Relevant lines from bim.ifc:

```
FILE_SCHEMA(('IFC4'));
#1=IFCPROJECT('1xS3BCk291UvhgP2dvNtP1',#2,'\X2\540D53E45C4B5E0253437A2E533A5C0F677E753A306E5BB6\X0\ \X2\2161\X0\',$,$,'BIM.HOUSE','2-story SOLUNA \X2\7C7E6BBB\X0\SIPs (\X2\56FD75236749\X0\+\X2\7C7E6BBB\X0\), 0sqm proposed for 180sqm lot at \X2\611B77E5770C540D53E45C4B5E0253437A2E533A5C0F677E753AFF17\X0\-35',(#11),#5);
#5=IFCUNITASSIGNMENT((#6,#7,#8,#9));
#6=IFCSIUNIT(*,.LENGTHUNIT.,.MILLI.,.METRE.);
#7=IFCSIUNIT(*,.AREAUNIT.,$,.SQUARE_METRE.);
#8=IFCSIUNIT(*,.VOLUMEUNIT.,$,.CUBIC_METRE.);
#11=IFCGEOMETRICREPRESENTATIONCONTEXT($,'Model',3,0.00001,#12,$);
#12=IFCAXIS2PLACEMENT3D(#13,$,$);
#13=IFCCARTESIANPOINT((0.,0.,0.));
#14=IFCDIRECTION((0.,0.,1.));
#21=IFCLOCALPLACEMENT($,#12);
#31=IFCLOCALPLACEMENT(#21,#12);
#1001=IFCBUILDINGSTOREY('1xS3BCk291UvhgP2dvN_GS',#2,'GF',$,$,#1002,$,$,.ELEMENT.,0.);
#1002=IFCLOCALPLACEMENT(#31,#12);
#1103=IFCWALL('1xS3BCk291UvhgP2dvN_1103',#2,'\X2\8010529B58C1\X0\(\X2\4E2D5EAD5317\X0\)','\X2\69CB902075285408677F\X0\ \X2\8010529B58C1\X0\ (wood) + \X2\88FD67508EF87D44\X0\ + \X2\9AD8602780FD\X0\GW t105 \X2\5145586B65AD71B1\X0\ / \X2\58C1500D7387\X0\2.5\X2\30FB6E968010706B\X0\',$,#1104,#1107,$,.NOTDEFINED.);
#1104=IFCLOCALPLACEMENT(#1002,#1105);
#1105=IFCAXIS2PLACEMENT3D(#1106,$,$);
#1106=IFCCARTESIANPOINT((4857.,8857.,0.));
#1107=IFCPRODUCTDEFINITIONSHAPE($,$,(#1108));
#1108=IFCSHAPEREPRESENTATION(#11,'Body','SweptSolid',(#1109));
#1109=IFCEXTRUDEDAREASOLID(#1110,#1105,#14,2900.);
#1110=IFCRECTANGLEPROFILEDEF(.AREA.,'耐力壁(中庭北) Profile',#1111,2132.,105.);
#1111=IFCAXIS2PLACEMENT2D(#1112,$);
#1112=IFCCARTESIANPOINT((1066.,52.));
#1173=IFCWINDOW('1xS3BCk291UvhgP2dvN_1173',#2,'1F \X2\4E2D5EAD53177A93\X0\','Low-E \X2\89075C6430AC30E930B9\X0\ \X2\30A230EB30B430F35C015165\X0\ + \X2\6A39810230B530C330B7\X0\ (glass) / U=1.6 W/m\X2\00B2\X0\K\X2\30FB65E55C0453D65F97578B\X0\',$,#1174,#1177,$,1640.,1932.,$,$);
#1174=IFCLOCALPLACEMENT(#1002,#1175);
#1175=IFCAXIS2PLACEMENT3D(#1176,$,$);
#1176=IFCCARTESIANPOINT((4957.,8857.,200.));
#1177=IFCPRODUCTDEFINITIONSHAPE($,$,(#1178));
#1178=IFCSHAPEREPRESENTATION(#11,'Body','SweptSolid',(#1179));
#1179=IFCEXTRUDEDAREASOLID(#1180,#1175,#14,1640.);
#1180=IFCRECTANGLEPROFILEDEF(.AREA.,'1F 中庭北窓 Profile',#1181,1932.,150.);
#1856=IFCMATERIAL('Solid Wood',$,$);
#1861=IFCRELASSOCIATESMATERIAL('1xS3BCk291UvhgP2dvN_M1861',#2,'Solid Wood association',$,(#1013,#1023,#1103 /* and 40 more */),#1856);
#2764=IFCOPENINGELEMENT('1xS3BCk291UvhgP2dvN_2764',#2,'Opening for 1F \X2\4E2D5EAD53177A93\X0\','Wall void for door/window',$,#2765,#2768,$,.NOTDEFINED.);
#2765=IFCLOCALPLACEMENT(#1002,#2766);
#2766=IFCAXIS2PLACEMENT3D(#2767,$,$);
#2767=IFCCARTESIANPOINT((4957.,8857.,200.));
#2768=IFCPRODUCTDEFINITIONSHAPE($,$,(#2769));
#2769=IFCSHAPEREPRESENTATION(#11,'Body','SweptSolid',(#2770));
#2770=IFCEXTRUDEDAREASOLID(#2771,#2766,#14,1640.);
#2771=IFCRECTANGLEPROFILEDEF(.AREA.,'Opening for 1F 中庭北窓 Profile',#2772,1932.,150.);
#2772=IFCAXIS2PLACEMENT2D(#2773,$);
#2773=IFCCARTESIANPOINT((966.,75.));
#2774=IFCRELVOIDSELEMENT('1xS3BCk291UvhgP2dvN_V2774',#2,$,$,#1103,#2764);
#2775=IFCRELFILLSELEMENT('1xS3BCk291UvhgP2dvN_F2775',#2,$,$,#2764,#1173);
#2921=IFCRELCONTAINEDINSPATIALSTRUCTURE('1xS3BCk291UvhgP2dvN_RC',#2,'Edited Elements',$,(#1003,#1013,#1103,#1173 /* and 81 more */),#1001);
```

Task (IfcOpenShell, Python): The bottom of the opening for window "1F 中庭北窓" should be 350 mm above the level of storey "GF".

```python
import numpy as np
import ifcopenshell
import ifcopenshell.api.geometry
import ifcopenshell.geom
import ifcopenshell.util.element
import ifcopenshell.util.placement
import ifcopenshell.util.shape
import ifcopenshell.util.unit

model = ifcopenshell.open("bim.ifc")
unit_scale = ifcopenshell.util.unit.calculate_unit_scale(model)

window = model.by_guid("1xS3BCk291UvhgP2dvN_1173")
opening = window.FillsVoids[0].RelatingOpeningElement
storey = ifcopenshell.util.element.get_container(window, ifc_class="IfcBuildingStorey")
level = ifcopenshell.util.placement.get_local_placement(storey.ObjectPlacement)[2, 3]

# The opening's origin need not be at the sill, so measure its lowest point.
shape = ifcopenshell.geom.create_shape(ifcopenshell.geom.settings(), opening)
bottom = ifcopenshell.util.shape.get_shape_bottom_elevation(shape, shape.geometry) / unit_scale
dz = level + 0.35 / unit_scale - bottom

shift = np.array([0.0, 0.0, dz])
# The window is not placed relative to its opening, so move both.
for product in (opening, window):
    matrix = ifcopenshell.util.placement.get_local_placement(product.ObjectPlacement)
    matrix[:3, 3] += shift
    ifcopenshell.api.geometry.edit_object_placement(model, product=product, matrix=matrix, is_si=False)

print(f"moved by {dz * unit_scale:+.3f} m")

model.write("bim_updated.ifc")
```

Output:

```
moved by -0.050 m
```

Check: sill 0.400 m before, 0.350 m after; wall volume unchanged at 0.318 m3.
